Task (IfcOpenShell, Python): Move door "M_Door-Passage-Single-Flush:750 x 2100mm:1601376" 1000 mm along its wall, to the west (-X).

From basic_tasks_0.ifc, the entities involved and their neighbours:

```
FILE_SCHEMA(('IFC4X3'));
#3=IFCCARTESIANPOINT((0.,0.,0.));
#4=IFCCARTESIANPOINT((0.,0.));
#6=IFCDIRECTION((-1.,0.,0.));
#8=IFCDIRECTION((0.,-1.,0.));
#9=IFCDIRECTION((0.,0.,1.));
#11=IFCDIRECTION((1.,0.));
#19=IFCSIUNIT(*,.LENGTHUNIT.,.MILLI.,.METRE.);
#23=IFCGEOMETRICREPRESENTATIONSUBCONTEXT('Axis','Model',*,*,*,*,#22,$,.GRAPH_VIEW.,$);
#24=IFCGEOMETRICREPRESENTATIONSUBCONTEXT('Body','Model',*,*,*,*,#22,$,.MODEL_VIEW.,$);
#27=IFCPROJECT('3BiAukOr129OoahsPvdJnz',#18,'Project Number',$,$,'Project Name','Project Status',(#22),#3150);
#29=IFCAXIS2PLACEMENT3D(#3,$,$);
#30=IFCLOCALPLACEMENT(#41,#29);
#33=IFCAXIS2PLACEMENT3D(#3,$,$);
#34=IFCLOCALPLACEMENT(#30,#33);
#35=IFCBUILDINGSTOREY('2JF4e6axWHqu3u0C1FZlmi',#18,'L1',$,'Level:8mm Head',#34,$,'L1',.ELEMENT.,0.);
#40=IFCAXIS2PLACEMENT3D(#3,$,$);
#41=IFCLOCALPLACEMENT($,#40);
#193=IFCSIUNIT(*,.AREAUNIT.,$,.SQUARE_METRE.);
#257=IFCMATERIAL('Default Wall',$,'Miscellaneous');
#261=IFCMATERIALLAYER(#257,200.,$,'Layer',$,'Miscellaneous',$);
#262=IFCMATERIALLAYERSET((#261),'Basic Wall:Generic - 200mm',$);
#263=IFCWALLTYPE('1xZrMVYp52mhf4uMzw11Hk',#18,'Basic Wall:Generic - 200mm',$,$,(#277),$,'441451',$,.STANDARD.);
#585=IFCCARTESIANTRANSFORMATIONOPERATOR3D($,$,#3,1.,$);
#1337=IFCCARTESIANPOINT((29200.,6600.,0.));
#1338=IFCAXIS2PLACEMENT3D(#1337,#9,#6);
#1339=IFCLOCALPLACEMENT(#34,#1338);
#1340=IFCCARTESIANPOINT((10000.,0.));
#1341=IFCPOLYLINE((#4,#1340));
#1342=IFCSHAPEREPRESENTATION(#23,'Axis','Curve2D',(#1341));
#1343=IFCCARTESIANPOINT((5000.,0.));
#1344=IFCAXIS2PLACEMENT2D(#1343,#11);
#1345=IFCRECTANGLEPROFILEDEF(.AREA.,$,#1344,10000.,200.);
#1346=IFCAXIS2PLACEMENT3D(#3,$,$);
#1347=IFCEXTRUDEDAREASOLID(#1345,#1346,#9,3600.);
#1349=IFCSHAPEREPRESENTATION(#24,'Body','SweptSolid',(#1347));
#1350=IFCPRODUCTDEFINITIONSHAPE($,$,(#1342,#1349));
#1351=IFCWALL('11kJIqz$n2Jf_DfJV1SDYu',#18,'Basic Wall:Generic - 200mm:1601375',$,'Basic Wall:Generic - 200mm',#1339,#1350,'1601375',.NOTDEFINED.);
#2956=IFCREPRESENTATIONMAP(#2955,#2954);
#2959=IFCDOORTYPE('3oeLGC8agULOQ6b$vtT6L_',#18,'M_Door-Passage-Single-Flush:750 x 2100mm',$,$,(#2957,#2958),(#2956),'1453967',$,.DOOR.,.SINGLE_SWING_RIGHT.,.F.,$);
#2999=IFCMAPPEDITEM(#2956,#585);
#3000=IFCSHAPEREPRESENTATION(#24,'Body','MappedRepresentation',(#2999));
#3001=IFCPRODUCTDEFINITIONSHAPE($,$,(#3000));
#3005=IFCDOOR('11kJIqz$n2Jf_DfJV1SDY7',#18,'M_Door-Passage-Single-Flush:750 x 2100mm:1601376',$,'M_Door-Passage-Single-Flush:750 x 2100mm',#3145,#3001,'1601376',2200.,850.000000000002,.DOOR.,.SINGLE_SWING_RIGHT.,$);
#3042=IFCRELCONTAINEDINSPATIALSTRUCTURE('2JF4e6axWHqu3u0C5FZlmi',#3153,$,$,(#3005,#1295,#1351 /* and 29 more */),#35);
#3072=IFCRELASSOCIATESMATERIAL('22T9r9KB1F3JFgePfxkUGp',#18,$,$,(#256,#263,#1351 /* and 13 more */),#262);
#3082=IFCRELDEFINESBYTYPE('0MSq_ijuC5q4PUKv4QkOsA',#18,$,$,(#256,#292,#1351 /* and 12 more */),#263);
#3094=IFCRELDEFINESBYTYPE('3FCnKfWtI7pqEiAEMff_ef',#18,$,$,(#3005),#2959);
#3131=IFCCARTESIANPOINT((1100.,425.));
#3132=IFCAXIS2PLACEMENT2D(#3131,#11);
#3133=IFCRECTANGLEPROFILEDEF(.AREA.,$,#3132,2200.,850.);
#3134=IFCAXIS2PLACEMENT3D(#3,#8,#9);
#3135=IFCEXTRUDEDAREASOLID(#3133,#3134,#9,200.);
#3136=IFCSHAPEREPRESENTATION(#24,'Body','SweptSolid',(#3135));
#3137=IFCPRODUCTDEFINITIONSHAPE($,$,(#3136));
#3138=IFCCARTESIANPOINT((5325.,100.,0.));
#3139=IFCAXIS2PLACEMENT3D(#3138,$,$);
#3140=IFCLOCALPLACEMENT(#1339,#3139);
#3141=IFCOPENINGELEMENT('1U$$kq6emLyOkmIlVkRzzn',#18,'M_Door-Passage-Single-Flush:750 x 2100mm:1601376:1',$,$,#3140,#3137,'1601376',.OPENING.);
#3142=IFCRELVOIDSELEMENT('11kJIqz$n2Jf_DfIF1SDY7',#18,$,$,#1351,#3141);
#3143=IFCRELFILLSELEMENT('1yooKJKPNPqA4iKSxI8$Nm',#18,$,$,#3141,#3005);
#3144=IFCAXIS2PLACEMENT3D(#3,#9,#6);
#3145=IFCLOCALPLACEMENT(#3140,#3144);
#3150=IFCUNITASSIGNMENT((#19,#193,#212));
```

```python
import ifcopenshell
import ifcopenshell.api.geometry
import ifcopenshell.util.placement

model = ifcopenshell.open("basic_tasks_0.ifc")

door = model.by_guid("11kJIqz$n2Jf_DfJV1SDY7")
opening = door.FillsVoids[0].RelatingOpeningElement
wall = opening.VoidsElements[0].RelatingBuildingElement

wall_matrix = ifcopenshell.util.placement.get_local_placement(wall.ObjectPlacement)
shift = wall_matrix[:3, 0] * 1000.0
before = ifcopenshell.util.placement.get_local_placement(door.ObjectPlacement)[:3, 3].copy()

# The door is placed relative to its opening, so it follows when the opening moves.
matrix = ifcopenshell.util.placement.get_local_placement(opening.ObjectPlacement)
matrix[:3, 3] += shift
ifcopenshell.api.geometry.edit_object_placement(
    model, product=opening, matrix=matrix, is_si=False, should_transform_children=True
)

after = ifcopenshell.util.placement.get_local_placement(door.ObjectPlacement)[:3, 3]
print("door moved by", (after - before).round(3) + 0.0)

model.write("basic_tasks_0_edited.ifc")
```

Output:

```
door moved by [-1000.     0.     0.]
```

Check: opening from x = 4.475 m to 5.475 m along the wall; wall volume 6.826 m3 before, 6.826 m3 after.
